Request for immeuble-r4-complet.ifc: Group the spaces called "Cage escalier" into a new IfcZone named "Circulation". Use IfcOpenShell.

First a look at what the model holds.

```python
import ifcopenshell

model = ifcopenshell.open("immeuble-r4-complet.ifc")
print(model.schema)
seen = {}
for space in model.by_type("IfcSpace"):
    seen[space.Name] = seen.get(space.Name, 0) + 1
for name, count in sorted(seen.items(), key=str):
    print(count, "x", name)
print("zones:", [z.Name for z in model.by_type("IfcZone")][:20])
```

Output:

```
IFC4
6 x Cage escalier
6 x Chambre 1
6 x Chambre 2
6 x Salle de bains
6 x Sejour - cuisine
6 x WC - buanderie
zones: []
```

```python
import ifcopenshell
import ifcopenshell.api.group
import ifcopenshell.api.root

model = ifcopenshell.open("immeuble-r4-complet.ifc")

names = {"Cage escalier"}
spaces = [s for s in model.by_type("IfcSpace") if s.Name in names]

zone = ifcopenshell.api.root.create_entity(model, ifc_class="IfcZone", name="Circulation")
ifcopenshell.api.group.assign_group(model, products=spaces, group=zone)
print(len(spaces), "spaces in", zone.Name)

model.write("immeuble-r4-complet_rev.ifc")
```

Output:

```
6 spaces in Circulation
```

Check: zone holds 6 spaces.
